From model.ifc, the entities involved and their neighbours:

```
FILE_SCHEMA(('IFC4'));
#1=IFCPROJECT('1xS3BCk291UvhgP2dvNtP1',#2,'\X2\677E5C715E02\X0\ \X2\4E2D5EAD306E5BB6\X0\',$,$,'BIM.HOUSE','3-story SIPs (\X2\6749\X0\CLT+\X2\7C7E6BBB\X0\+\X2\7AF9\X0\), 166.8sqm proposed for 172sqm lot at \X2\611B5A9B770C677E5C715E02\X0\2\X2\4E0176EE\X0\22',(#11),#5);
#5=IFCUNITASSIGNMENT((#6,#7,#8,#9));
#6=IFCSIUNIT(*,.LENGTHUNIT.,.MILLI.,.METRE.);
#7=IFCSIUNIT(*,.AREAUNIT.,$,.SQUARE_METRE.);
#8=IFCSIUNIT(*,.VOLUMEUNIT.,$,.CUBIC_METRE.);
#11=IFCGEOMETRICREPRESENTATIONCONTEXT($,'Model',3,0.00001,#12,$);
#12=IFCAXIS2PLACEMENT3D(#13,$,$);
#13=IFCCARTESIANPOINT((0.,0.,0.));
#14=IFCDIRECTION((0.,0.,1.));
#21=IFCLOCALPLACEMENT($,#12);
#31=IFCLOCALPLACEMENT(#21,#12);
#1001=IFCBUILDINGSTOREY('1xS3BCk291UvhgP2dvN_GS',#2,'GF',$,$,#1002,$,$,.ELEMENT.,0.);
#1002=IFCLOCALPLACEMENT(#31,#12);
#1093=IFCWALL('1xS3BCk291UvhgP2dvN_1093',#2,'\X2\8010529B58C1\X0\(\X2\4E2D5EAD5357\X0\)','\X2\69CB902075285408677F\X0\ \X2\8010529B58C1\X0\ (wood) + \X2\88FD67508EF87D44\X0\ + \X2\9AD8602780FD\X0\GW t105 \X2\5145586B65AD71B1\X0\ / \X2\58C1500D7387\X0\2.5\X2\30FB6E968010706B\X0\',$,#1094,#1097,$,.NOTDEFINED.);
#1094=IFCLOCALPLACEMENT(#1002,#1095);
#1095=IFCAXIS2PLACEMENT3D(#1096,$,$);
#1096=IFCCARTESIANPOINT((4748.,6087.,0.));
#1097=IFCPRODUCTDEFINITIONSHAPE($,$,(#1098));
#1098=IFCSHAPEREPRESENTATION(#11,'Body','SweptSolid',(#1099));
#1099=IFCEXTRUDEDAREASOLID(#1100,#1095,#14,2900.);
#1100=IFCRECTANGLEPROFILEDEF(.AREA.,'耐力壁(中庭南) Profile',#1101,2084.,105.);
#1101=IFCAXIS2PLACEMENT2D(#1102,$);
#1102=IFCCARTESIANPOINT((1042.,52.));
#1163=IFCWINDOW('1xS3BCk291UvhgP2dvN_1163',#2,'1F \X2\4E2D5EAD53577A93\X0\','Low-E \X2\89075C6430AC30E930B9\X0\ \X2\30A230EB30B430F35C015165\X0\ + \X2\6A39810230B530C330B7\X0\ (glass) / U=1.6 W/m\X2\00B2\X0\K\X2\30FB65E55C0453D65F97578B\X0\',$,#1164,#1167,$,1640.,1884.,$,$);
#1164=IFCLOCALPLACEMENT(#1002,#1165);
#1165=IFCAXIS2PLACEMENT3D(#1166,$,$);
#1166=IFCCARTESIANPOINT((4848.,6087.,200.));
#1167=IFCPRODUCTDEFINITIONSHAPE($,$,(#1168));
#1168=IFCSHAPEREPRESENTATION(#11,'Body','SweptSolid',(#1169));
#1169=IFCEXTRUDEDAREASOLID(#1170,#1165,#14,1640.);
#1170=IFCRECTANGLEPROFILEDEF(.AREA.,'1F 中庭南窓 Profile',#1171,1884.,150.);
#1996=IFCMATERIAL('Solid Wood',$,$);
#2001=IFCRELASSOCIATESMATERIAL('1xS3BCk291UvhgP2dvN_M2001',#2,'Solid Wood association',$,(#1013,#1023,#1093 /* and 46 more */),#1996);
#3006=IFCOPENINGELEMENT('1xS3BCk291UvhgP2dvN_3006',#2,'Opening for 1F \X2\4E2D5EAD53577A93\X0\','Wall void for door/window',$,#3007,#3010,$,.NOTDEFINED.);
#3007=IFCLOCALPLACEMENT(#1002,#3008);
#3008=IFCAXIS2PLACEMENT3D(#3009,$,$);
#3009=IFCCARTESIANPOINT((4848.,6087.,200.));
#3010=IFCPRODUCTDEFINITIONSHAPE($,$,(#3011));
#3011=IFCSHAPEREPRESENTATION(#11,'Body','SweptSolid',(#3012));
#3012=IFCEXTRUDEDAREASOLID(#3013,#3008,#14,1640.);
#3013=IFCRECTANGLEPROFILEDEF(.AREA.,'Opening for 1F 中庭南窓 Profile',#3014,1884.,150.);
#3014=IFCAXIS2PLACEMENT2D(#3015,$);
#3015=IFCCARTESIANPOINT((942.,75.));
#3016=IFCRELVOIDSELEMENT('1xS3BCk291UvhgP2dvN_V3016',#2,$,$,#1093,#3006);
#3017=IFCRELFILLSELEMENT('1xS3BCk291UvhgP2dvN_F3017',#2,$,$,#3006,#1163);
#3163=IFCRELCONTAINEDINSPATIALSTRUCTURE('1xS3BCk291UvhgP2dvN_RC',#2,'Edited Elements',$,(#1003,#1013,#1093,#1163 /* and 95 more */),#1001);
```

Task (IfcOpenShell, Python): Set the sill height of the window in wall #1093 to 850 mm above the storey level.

```python
import numpy as np
import ifcopenshell
import ifcopenshell.api.geometry
import ifcopenshell.geom
import ifcopenshell.util.element
import ifcopenshell.util.placement
import ifcopenshell.util.shape
import ifcopenshell.util.unit

model = ifcopenshell.open("model.ifc")
unit_scale = ifcopenshell.util.unit.calculate_unit_scale(model)

window = model.by_id(1163)
opening = window.FillsVoids[0].RelatingOpeningElement
storey = ifcopenshell.util.element.get_container(window, ifc_class="IfcBuildingStorey")
level = ifcopenshell.util.placement.get_local_placement(storey.ObjectPlacement)[2, 3]

# The opening's origin need not be at the sill, so measure its lowest point.
shape = ifcopenshell.geom.create_shape(ifcopenshell.geom.settings(), opening)
bottom = ifcopenshell.util.shape.get_shape_bottom_elevation(shape, shape.geometry) / unit_scale
dz = level + 850.0 - bottom

shift = np.array([0.0, 0.0, dz])
# The window is not placed relative to its opening, so move both.
for product in (opening, window):
    matrix = ifcopenshell.util.placement.get_local_placement(product.ObjectPlacement)
    matrix[:3, 3] += shift
    ifcopenshell.api.geometry.edit_object_placement(model, product=product, matrix=matrix, is_si=False)

print(f"moved by {dz * unit_scale:+.3f} m")

model.write("model-out.ifc")
```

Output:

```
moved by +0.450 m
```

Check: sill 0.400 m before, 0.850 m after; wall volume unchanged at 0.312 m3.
